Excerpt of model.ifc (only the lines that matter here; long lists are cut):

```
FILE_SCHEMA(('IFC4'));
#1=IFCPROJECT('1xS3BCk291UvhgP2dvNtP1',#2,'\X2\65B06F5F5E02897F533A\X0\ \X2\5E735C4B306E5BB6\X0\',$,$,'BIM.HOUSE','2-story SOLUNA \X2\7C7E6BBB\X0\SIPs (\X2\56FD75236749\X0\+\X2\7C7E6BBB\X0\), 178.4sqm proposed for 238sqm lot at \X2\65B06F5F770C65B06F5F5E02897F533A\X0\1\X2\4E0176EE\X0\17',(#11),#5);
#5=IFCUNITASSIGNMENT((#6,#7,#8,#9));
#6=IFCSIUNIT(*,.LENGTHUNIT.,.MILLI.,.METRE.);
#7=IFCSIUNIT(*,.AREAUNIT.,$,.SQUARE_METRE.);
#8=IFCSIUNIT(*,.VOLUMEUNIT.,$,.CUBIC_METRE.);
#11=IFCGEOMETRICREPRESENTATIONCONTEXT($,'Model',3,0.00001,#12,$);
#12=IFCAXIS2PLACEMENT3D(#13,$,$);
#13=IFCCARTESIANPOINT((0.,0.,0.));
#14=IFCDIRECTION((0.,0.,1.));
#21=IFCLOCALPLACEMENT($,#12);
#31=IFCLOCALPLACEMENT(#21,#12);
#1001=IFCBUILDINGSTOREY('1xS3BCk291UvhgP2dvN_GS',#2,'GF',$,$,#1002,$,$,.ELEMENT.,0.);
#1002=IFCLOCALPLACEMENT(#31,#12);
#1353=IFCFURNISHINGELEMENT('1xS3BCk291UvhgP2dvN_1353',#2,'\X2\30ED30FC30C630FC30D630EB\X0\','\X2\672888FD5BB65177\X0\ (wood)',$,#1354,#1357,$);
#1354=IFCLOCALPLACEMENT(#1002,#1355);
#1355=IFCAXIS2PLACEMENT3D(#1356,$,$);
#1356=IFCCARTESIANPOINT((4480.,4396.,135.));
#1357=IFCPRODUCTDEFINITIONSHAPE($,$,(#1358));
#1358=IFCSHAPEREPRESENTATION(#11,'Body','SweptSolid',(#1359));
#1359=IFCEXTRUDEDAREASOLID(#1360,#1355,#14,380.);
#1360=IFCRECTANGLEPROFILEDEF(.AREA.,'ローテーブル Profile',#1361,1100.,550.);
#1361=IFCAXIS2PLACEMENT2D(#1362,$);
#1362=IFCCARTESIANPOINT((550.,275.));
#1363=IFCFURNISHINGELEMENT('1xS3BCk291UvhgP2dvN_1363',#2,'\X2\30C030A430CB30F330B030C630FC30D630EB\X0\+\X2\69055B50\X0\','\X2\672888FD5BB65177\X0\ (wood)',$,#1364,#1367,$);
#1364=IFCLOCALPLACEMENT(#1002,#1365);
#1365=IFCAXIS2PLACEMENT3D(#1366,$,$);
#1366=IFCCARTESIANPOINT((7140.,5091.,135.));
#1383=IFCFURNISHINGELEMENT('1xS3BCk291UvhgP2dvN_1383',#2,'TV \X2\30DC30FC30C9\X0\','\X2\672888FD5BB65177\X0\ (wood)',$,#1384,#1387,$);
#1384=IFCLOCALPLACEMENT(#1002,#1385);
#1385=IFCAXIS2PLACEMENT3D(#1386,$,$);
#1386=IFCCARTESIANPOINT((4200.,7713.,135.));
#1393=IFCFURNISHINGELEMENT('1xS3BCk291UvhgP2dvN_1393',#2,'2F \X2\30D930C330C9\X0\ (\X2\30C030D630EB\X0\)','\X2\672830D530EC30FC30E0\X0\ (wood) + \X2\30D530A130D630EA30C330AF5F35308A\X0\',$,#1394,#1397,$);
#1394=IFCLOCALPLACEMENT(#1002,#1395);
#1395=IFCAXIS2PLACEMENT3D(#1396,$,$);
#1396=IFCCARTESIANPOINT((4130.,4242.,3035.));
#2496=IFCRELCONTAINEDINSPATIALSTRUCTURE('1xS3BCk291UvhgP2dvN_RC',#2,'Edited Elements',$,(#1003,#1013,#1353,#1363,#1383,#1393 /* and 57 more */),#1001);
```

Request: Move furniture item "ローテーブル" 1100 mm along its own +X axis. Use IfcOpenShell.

```python
import ifcopenshell
import ifcopenshell.api.geometry
import ifcopenshell.util.placement

model = ifcopenshell.open("model.ifc")

item = model.by_id(1353)
matrix = ifcopenshell.util.placement.get_local_placement(item.ObjectPlacement)
matrix[:3, 3] += matrix[:3, 0] * 1100.0
ifcopenshell.api.geometry.edit_object_placement(model, product=item, matrix=matrix, is_si=False)

print(ifcopenshell.util.placement.get_local_placement(item.ObjectPlacement).round(3) + 0.0)

model.write("model_updated.ifc")
```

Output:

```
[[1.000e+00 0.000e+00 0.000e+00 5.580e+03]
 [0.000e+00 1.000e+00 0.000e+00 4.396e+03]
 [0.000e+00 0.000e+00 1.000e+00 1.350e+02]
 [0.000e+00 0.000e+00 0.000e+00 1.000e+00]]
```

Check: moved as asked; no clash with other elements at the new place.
